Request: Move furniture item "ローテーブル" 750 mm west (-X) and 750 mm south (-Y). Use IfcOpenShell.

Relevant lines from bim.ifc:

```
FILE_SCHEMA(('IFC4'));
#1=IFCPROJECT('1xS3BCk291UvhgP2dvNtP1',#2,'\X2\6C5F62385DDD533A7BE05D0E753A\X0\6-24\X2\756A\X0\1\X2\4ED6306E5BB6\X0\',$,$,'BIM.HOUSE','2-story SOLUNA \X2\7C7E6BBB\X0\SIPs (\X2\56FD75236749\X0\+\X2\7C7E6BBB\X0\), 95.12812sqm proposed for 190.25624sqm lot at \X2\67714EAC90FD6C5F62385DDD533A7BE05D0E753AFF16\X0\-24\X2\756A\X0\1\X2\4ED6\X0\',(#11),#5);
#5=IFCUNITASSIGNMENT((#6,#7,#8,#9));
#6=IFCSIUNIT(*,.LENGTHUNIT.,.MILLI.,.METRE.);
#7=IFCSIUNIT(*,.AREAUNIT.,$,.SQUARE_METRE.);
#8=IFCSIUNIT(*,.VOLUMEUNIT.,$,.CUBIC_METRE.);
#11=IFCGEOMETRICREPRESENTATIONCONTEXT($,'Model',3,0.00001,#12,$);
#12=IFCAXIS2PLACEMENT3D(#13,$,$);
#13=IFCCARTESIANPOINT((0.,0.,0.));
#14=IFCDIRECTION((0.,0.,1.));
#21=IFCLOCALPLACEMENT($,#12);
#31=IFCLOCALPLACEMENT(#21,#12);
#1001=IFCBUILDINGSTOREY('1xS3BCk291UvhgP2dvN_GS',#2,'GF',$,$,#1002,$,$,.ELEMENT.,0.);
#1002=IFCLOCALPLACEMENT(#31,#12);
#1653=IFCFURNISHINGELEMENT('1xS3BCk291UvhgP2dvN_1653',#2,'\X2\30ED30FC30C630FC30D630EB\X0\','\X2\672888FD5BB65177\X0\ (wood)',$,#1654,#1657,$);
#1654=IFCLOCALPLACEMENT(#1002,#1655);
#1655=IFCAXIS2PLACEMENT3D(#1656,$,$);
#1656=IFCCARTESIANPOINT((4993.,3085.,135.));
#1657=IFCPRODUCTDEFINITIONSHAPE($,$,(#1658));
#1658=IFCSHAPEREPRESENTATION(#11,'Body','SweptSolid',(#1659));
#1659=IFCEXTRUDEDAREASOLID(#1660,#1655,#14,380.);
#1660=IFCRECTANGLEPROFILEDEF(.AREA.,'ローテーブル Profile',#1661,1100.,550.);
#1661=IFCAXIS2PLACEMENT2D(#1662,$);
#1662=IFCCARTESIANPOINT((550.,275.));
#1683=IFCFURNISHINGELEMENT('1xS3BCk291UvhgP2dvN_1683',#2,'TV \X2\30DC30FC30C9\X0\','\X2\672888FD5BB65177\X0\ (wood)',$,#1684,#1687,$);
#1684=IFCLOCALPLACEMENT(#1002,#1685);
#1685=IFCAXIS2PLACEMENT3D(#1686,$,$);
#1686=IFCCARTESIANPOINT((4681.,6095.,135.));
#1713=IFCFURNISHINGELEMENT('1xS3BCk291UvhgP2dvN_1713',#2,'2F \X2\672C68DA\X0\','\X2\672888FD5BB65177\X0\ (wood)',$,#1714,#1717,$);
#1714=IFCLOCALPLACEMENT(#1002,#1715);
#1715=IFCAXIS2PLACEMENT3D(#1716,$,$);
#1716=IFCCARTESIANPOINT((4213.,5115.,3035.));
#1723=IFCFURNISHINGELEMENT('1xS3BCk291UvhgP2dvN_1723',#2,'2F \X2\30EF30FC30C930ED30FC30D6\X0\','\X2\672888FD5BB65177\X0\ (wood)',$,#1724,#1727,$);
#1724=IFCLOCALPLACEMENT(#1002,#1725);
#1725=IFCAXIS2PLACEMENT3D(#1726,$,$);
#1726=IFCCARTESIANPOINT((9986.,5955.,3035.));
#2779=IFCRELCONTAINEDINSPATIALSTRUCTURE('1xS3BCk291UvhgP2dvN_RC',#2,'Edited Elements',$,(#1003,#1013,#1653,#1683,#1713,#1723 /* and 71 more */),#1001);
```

```python
import ifcopenshell
import ifcopenshell.api.geometry
import ifcopenshell.util.placement

model = ifcopenshell.open("bim.ifc")

item = model.by_id(1653)
matrix = ifcopenshell.util.placement.get_local_placement(item.ObjectPlacement)
matrix[0, 3] -= 750.0
matrix[1, 3] -= 750.0
ifcopenshell.api.geometry.edit_object_placement(model, product=item, matrix=matrix, is_si=False)

print(ifcopenshell.util.placement.get_local_placement(item.ObjectPlacement).round(3) + 0.0)

model.write("bim_rev.ifc")
```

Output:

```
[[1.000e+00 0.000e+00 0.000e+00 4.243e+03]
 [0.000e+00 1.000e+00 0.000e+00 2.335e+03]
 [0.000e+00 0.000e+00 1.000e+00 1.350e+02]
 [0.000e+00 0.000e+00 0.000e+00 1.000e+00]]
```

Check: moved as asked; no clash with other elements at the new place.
